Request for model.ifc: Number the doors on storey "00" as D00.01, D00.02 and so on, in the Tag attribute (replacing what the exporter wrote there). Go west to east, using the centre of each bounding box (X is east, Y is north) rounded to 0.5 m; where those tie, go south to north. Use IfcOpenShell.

First a look at what the model holds.

```python
import ifcopenshell
import ifcopenshell.util.element
import ifcopenshell.util.placement

model = ifcopenshell.open("model.ifc")
print(model.schema)
storey = next(s for s in model.by_type("IfcBuildingStorey") if s.Name == "00")
doors = [e for e in ifcopenshell.util.element.get_decomposition(storey) if e.is_a("IfcDoor")]
for e in sorted(doors, key=lambda e: e.id()):
    origin = ifcopenshell.util.placement.get_local_placement(e.ObjectPlacement)[:3, 3]
    print(e.id(), e.Tag, e.Name, origin.round(2) + 0.0, sep=" | ")
```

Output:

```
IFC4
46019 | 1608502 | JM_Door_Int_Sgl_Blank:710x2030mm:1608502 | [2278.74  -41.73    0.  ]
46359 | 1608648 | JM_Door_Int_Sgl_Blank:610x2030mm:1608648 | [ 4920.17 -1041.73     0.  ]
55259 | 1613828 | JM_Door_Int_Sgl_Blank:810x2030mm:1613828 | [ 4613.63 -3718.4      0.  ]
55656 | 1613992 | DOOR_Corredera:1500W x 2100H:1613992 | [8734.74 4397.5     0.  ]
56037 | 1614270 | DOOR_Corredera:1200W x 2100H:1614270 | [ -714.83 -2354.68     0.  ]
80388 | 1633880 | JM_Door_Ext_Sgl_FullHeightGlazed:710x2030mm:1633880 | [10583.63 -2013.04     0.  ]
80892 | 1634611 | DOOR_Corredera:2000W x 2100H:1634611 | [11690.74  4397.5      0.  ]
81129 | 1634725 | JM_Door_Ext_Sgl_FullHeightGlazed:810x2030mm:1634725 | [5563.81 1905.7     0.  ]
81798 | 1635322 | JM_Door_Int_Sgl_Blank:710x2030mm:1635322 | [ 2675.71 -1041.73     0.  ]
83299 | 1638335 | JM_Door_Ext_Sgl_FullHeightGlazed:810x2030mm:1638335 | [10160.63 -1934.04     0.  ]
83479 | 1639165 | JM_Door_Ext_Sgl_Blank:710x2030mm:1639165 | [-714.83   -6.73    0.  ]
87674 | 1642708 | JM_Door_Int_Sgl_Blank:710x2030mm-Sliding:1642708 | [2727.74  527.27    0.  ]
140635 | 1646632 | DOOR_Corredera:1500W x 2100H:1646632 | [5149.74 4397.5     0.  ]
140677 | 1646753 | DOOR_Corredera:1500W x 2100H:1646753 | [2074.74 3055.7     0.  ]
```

```python
import ifcopenshell
import ifcopenshell.geom
import ifcopenshell.util.element
import ifcopenshell.util.shape

model = ifcopenshell.open("model.ifc")
settings = ifcopenshell.geom.settings()
settings.set("use-world-coords", True)


def centre(element):
    shape = ifcopenshell.geom.create_shape(settings, element)
    return ifcopenshell.util.shape.get_bbox_centroid(shape.geometry)


storey = next(s for s in model.by_type("IfcBuildingStorey") if s.Name == "00")
doors = [e for e in ifcopenshell.util.element.get_decomposition(storey) if e.is_a("IfcDoor")]

# Insertion points can sit at a corner or the storey origin, so sort by the geometry (in metres).
centres = {e: centre(e) for e in doors}
doors.sort(key=lambda e: (round(centres[e][0] / 0.5), centres[e][1]))

for i, e in enumerate(doors, start=1):
    number = f"D00.{i:02d}"
    e.Tag = number
    print(e.id(), number)

model.write("model_updated.ifc")
```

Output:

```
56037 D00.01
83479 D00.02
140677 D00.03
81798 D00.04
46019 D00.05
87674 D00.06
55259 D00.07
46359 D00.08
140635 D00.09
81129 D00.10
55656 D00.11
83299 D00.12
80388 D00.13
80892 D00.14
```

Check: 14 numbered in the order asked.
